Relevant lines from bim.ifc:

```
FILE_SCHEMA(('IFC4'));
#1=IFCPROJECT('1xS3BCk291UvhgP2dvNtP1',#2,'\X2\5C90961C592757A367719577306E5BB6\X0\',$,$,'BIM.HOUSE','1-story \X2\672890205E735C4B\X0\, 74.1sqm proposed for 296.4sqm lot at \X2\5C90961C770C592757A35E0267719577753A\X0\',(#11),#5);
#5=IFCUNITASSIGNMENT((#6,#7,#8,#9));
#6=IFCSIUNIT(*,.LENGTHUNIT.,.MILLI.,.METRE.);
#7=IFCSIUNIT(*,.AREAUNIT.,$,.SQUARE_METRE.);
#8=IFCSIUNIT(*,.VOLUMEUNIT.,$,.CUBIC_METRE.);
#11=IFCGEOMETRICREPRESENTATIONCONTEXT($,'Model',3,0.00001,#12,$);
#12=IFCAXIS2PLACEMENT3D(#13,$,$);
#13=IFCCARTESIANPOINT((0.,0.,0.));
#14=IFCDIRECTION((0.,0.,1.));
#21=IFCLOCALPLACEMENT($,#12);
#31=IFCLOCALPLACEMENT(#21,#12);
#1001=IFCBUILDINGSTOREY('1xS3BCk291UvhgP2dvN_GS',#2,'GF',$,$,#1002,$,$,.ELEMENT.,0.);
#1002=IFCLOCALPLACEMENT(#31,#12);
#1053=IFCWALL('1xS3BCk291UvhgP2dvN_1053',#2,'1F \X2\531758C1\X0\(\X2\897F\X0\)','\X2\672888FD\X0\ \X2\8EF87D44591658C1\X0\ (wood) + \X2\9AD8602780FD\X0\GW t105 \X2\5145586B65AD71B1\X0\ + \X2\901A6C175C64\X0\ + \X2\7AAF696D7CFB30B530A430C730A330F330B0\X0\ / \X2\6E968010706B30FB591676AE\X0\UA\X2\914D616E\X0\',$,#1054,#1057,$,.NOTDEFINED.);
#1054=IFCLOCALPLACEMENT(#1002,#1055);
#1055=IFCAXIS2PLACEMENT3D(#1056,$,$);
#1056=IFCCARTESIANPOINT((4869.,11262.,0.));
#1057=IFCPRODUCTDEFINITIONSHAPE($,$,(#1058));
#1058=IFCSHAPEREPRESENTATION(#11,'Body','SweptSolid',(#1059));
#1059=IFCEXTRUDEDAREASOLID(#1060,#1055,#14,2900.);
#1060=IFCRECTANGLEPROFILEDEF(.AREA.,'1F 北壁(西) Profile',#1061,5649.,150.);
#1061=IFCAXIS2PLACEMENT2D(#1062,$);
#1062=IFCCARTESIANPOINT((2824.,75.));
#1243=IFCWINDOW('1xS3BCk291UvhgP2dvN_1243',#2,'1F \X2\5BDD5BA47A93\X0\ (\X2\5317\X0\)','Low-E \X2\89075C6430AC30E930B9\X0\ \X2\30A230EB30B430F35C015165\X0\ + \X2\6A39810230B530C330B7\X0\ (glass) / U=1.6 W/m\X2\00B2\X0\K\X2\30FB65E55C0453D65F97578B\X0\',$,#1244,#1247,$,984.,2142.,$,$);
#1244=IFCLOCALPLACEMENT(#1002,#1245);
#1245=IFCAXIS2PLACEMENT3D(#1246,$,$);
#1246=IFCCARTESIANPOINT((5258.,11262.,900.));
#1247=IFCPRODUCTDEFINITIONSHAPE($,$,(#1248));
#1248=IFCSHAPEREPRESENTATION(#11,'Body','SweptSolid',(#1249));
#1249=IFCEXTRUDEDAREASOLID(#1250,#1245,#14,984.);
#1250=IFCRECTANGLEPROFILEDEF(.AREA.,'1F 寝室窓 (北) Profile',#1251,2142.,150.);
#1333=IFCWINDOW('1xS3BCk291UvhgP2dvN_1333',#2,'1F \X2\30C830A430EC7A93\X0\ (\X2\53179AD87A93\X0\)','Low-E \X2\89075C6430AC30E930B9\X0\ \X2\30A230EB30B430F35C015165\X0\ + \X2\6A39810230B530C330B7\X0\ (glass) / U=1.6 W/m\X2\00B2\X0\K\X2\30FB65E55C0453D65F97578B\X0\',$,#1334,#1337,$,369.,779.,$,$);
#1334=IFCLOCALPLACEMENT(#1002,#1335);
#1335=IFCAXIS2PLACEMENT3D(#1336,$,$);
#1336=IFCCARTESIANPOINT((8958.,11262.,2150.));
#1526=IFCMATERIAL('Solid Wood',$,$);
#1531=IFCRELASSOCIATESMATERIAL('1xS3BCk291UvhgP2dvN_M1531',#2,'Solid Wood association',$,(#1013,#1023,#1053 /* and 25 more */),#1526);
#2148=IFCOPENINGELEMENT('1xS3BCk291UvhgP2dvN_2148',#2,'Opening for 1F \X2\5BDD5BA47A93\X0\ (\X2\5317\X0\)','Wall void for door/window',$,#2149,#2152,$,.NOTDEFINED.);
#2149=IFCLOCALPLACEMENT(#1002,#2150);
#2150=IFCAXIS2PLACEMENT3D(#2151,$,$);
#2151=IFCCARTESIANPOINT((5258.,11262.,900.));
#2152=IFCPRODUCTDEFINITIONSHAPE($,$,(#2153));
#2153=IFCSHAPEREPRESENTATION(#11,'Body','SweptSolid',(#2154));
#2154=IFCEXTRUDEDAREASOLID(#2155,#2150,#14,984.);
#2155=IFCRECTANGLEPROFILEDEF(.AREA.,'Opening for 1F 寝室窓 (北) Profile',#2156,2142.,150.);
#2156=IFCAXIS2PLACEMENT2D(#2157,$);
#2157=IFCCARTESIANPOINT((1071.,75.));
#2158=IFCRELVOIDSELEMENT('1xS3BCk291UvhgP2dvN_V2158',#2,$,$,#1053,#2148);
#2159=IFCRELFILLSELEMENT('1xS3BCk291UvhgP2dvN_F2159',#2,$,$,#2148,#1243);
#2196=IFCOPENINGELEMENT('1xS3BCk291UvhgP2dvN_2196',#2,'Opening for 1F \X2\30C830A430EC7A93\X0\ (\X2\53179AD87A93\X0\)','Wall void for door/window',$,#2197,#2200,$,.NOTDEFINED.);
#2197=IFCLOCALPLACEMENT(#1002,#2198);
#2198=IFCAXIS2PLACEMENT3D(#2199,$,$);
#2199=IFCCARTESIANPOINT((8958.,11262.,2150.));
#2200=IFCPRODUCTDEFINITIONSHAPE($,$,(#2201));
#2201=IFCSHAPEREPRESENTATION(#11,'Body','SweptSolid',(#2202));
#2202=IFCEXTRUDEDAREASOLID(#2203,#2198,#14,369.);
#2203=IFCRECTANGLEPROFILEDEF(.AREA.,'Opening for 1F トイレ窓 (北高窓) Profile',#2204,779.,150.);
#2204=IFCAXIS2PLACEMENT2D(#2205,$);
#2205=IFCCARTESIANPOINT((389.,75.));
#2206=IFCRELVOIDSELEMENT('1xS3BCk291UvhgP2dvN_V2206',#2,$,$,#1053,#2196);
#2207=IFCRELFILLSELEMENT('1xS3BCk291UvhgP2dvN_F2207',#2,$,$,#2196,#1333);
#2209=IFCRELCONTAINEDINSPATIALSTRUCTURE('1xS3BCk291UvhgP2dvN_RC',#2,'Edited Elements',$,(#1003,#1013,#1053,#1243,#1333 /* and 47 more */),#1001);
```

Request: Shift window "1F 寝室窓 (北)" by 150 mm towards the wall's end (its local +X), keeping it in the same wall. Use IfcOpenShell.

```python
import ifcopenshell
import ifcopenshell.api.geometry
import ifcopenshell.util.placement

model = ifcopenshell.open("bim.ifc")

window = model.by_id(1243)
opening = window.FillsVoids[0].RelatingOpeningElement
wall = opening.VoidsElements[0].RelatingBuildingElement

wall_matrix = ifcopenshell.util.placement.get_local_placement(wall.ObjectPlacement)
shift = wall_matrix[:3, 0] * 150.0
before = ifcopenshell.util.placement.get_local_placement(window.ObjectPlacement)[:3, 3].copy()

# The window is not placed relative to its opening, so move both.
for product in (opening, window):
    matrix = ifcopenshell.util.placement.get_local_placement(product.ObjectPlacement)
    matrix[:3, 3] += shift
    ifcopenshell.api.geometry.edit_object_placement(model, product=product, matrix=matrix, is_si=False)

after = ifcopenshell.util.placement.get_local_placement(window.ObjectPlacement)[:3, 3]
print("window moved by", (after - before).round(3) + 0.0)

model.write("bim_updated.ifc")
```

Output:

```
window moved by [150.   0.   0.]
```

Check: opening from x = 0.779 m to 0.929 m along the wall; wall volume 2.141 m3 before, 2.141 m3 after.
